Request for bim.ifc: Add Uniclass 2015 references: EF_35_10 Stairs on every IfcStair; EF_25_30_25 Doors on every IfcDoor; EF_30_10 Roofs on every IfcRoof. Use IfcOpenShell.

First a look at what the model holds.

```python
import ifcopenshell

model = ifcopenshell.open("bim.ifc")
print(model.schema)
print("classifications:", [c.Name for c in model.by_type("IfcClassification")])
for ifc_class in ("IfcDoor", "IfcRoof", "IfcStair", "IfcWall", "IfcWindow"):
    print(ifc_class, len(model.by_type(ifc_class)))
```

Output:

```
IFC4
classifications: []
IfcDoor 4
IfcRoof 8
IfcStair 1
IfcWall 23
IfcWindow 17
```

```python
import ifcopenshell
import ifcopenshell.api.classification

model = ifcopenshell.open("bim.ifc")

system = ifcopenshell.api.classification.add_classification(model, classification="Uniclass 2015")

codes = {
    "IfcStair": ("EF_35_10", "Stairs"),
    "IfcDoor": ("EF_25_30_25", "Doors"),
    "IfcRoof": ("EF_30_10", "Roofs"),
}
for ifc_class, (code, name) in codes.items():
    products = model.by_type(ifc_class)
    ifcopenshell.api.classification.add_reference(
        model, products=products, classification=system, identification=code, name=name
    )
    print(code, len(products))

model.write("bim_updated.ifc")
```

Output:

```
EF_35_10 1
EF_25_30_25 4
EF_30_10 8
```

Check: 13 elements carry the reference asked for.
